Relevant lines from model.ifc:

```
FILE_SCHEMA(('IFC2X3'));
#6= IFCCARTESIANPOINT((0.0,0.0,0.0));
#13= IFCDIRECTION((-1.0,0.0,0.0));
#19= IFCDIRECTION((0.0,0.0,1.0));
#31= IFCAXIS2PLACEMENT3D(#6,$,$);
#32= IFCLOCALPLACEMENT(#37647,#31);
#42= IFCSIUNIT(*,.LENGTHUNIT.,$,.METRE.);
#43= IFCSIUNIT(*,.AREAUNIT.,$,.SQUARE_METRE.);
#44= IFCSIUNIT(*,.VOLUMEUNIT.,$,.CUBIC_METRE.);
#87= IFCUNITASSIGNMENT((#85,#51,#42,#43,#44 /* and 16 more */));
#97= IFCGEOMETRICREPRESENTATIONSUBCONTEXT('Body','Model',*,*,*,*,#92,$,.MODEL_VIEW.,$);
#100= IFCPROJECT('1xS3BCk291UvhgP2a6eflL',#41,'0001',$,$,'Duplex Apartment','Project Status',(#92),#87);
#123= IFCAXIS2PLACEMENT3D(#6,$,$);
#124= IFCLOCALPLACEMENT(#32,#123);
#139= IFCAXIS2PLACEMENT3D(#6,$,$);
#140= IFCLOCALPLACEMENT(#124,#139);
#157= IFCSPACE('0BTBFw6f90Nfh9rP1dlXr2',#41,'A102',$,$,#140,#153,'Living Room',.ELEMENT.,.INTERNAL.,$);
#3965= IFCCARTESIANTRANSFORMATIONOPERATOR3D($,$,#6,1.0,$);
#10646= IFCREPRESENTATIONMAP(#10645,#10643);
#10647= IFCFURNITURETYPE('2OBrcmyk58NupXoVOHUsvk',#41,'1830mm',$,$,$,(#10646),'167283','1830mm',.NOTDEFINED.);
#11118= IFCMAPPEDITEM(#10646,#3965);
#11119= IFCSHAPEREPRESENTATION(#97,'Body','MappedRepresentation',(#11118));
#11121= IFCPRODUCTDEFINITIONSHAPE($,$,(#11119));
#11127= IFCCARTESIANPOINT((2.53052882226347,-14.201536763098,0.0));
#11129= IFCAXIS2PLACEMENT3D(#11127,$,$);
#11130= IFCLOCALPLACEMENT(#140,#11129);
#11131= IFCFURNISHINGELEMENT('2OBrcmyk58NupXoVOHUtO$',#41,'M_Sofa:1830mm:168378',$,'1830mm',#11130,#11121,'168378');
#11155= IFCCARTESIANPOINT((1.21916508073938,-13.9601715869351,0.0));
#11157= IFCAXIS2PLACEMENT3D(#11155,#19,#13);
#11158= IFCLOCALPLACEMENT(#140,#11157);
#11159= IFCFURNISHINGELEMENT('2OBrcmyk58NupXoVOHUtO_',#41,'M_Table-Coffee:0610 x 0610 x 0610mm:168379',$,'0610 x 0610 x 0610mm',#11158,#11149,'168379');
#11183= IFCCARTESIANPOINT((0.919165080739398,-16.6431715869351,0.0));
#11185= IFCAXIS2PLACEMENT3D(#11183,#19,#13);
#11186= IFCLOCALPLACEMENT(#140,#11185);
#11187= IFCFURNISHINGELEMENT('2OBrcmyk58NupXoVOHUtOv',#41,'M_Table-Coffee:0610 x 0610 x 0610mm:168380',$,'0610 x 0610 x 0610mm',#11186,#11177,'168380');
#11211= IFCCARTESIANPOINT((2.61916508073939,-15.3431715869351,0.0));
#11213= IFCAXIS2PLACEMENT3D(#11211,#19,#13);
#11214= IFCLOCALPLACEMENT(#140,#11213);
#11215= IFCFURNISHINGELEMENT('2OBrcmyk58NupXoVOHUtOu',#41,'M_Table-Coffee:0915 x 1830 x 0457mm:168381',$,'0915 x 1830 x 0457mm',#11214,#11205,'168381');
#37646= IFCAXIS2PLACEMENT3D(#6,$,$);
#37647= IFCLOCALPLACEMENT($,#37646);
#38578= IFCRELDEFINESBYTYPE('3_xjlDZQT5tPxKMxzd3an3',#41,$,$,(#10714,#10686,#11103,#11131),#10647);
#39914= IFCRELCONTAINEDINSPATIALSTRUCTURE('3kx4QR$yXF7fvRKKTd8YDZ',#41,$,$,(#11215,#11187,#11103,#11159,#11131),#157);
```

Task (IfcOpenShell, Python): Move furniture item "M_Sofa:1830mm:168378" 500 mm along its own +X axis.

```python
import ifcopenshell
import ifcopenshell.api.geometry
import ifcopenshell.util.placement

model = ifcopenshell.open("model.ifc")

item = model.by_guid("2OBrcmyk58NupXoVOHUtO$")
matrix = ifcopenshell.util.placement.get_local_placement(item.ObjectPlacement)
matrix[:3, 3] += matrix[:3, 0] * 0.5
ifcopenshell.api.geometry.edit_object_placement(model, product=item, matrix=matrix, is_si=False)

print(ifcopenshell.util.placement.get_local_placement(item.ObjectPlacement).round(3) + 0.0)

model.write("model_v2.ifc")
```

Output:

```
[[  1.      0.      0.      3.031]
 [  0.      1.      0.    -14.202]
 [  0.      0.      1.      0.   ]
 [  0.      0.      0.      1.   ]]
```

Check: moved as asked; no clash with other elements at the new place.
